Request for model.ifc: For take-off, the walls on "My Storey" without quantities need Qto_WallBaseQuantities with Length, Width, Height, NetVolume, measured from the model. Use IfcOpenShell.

First a look at what the model holds.

```python
import ifcopenshell
import ifcopenshell.util.element
import ifcopenshell.util.unit

model = ifcopenshell.open("model.ifc")
print(model.schema)
for unit_type in ("LENGTHUNIT", "AREAUNIT", "VOLUMEUNIT"):
    print(unit_type, ifcopenshell.util.unit.calculate_unit_scale(model, unit_type))
storey = next(s for s in model.by_type("IfcBuildingStorey") if s.Name == "My Storey")
walls = [e for e in ifcopenshell.util.element.get_decomposition(storey) if e.is_a("IfcWall")]
for e in sorted(walls, key=lambda e: e.id()):
    print(e.id(), e.is_a(), e.Name, list(ifcopenshell.util.element.get_psets(e, qtos_only=True)), sep=" | ")
```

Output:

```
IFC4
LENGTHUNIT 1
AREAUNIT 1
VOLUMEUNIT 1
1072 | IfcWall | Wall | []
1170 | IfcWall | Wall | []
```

```python
import ifcopenshell
import ifcopenshell.api.pset
import ifcopenshell.geom
import ifcopenshell.util.element
import ifcopenshell.util.shape
import ifcopenshell.util.unit

model = ifcopenshell.open("model.ifc")
unit_scale = ifcopenshell.util.unit.calculate_unit_scale(model)
volume_scale = ifcopenshell.util.unit.calculate_unit_scale(model, "VOLUMEUNIT")
settings = ifcopenshell.geom.settings()

storey = next(s for s in model.by_type("IfcBuildingStorey") if s.Name == "My Storey")
walls = [e for e in ifcopenshell.util.element.get_decomposition(storey) if e.is_a("IfcWall")]

for e in sorted(walls, key=lambda e: e.id()):
    if ifcopenshell.util.element.get_psets(e, qtos_only=True, should_inherit=False):
        continue
    # Geometry comes back in metres, in the element's own axes.
    shape = ifcopenshell.geom.create_shape(settings, e)
    values = {
        "Length": ifcopenshell.util.shape.get_x(shape.geometry) / unit_scale,
        "Width": ifcopenshell.util.shape.get_y(shape.geometry) / unit_scale,
        "Height": ifcopenshell.util.shape.get_z(shape.geometry) / unit_scale,
        "NetVolume": ifcopenshell.util.shape.get_volume(shape.geometry) / volume_scale,
    }
    qto = ifcopenshell.api.pset.add_qto(model, product=e, name="Qto_WallBaseQuantities")
    ifcopenshell.api.pset.edit_qto(model, qto=qto, properties=values)
    print(e.id(), {k: round(v, 3) for k, v in values.items()})

model.write("model-out.ifc")
```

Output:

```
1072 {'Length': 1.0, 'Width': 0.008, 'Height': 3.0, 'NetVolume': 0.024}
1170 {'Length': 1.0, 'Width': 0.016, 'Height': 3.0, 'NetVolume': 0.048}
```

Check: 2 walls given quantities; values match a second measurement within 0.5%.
